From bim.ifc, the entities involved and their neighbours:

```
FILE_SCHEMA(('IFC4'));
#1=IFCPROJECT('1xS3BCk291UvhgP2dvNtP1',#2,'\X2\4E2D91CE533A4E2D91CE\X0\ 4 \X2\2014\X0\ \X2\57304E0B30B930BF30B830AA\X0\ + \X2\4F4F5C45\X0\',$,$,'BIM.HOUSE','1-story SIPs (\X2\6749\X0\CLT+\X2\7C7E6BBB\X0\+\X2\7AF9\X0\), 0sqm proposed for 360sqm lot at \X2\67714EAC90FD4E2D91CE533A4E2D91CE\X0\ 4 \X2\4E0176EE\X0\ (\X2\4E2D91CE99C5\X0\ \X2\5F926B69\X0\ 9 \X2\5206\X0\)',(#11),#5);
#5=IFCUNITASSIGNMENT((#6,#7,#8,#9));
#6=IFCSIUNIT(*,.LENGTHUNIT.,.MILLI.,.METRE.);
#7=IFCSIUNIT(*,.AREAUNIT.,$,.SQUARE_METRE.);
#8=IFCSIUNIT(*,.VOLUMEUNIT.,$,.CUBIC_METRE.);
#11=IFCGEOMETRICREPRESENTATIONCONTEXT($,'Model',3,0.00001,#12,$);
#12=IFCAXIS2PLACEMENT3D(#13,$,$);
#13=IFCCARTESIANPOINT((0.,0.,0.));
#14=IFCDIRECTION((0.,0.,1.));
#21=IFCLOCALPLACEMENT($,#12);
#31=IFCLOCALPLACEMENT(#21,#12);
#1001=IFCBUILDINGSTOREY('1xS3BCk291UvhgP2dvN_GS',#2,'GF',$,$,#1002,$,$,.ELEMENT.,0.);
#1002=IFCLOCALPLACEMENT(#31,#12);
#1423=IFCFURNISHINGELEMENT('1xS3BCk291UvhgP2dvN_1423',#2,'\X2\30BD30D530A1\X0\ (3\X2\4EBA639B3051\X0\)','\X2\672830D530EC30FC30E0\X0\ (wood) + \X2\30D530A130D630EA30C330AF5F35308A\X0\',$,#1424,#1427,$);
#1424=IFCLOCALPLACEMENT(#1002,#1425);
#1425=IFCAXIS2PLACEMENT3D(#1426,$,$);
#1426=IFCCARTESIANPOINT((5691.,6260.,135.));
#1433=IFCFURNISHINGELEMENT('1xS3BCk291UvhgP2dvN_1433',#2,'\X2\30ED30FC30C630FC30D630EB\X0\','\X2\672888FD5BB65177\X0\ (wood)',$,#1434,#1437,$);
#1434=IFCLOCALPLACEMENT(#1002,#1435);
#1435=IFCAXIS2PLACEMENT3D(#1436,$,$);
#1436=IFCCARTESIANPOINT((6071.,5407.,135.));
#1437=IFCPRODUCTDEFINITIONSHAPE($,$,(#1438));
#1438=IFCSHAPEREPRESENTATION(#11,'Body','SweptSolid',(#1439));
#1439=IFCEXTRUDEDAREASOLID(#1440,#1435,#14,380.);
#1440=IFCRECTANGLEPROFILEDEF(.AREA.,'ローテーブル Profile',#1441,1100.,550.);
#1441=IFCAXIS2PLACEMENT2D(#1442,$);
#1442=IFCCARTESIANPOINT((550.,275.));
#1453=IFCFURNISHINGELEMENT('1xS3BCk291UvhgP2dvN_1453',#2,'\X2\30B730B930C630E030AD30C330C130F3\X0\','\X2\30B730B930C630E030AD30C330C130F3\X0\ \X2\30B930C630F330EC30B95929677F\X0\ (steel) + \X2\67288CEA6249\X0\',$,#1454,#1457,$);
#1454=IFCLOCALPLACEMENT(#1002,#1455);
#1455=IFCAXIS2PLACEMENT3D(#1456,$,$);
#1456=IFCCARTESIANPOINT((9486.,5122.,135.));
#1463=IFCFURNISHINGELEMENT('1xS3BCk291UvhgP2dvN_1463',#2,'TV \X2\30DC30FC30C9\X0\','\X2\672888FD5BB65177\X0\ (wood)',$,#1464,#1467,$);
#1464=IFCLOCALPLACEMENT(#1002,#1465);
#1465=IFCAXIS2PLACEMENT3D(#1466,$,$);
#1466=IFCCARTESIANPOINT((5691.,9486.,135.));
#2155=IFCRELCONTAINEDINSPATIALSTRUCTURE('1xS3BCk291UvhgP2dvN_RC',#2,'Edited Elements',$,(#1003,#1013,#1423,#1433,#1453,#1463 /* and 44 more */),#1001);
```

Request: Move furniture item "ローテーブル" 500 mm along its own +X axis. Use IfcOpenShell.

```python
import ifcopenshell
import ifcopenshell.api.geometry
import ifcopenshell.util.placement
import ifcopenshell.util.unit

model = ifcopenshell.open("bim.ifc")
unit_scale = ifcopenshell.util.unit.calculate_unit_scale(model)

item = model.by_id(1433)
matrix = ifcopenshell.util.placement.get_local_placement(item.ObjectPlacement)
matrix[:3, 3] += matrix[:3, 0] * 0.5 / unit_scale
ifcopenshell.api.geometry.edit_object_placement(model, product=item, matrix=matrix, is_si=False)

print(ifcopenshell.util.placement.get_local_placement(item.ObjectPlacement).round(3) + 0.0)

model.write("bim_edited.ifc")
```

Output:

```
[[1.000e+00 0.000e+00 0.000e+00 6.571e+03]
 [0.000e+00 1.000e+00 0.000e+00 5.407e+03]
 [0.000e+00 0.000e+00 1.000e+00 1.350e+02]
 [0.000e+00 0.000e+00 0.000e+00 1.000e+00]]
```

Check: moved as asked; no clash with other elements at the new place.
